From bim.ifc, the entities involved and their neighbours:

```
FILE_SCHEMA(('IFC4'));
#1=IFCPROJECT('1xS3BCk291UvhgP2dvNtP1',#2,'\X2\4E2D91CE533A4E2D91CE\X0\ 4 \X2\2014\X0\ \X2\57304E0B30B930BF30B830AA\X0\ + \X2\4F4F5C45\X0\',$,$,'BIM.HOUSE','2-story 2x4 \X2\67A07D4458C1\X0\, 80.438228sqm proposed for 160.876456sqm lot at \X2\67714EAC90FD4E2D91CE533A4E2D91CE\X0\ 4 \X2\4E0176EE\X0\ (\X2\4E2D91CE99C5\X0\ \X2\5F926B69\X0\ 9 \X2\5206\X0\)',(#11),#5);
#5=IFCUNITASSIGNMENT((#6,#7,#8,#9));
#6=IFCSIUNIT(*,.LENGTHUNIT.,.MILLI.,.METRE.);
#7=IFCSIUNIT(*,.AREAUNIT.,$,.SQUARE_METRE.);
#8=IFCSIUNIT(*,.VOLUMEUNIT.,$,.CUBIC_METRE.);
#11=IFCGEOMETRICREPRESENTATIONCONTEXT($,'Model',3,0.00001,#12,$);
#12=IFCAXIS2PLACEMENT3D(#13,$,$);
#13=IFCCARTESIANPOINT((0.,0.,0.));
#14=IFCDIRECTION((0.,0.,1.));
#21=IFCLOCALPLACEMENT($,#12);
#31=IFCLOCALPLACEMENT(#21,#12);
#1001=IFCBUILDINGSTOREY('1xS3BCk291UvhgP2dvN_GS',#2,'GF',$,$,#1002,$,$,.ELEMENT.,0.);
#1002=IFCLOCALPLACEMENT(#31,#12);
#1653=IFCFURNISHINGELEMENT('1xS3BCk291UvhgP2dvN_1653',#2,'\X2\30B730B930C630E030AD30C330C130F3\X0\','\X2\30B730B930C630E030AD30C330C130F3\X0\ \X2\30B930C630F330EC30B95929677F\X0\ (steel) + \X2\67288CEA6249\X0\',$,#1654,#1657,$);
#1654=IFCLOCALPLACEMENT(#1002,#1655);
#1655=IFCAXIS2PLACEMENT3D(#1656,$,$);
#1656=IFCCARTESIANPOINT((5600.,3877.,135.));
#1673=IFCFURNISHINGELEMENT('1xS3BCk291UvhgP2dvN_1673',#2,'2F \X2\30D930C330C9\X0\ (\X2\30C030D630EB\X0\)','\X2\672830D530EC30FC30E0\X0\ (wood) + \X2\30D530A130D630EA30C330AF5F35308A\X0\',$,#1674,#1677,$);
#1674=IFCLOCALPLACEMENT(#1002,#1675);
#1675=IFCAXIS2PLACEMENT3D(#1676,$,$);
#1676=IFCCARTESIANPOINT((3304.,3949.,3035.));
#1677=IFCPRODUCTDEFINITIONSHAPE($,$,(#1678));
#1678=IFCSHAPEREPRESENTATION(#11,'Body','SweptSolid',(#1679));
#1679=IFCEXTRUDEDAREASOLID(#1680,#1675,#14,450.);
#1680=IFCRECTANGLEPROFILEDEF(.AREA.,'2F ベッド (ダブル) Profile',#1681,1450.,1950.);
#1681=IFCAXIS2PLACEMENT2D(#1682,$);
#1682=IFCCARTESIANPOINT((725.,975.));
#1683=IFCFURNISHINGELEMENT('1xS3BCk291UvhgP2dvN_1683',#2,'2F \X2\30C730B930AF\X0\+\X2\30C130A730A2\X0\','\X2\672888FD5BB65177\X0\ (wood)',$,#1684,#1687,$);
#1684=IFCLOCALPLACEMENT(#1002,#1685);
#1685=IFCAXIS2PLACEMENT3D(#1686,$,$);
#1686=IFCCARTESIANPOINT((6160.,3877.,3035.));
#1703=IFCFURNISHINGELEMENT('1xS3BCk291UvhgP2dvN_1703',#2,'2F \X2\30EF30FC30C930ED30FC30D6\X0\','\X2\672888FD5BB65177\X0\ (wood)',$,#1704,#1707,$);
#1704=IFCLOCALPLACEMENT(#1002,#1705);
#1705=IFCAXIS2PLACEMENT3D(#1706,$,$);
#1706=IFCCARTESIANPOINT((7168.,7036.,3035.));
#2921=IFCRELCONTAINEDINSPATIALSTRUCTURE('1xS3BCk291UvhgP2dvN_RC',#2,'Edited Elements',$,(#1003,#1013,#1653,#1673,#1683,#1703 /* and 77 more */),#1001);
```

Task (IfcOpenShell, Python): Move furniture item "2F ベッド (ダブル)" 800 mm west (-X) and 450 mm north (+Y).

```python
import ifcopenshell
import ifcopenshell.api.geometry
import ifcopenshell.util.placement
import ifcopenshell.util.unit

model = ifcopenshell.open("bim.ifc")
unit_scale = ifcopenshell.util.unit.calculate_unit_scale(model)

item = model.by_guid("1xS3BCk291UvhgP2dvN_1673")
matrix = ifcopenshell.util.placement.get_local_placement(item.ObjectPlacement)
matrix[0, 3] -= 0.8 / unit_scale
matrix[1, 3] += 0.45 / unit_scale
ifcopenshell.api.geometry.edit_object_placement(model, product=item, matrix=matrix, is_si=False)

print(ifcopenshell.util.placement.get_local_placement(item.ObjectPlacement).round(3) + 0.0)

model.write("bim_edited.ifc")
```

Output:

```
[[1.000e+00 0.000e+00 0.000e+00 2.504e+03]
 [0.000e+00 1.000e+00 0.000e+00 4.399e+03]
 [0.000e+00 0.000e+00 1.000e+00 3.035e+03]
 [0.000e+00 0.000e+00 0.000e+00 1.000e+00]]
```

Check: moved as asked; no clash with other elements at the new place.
